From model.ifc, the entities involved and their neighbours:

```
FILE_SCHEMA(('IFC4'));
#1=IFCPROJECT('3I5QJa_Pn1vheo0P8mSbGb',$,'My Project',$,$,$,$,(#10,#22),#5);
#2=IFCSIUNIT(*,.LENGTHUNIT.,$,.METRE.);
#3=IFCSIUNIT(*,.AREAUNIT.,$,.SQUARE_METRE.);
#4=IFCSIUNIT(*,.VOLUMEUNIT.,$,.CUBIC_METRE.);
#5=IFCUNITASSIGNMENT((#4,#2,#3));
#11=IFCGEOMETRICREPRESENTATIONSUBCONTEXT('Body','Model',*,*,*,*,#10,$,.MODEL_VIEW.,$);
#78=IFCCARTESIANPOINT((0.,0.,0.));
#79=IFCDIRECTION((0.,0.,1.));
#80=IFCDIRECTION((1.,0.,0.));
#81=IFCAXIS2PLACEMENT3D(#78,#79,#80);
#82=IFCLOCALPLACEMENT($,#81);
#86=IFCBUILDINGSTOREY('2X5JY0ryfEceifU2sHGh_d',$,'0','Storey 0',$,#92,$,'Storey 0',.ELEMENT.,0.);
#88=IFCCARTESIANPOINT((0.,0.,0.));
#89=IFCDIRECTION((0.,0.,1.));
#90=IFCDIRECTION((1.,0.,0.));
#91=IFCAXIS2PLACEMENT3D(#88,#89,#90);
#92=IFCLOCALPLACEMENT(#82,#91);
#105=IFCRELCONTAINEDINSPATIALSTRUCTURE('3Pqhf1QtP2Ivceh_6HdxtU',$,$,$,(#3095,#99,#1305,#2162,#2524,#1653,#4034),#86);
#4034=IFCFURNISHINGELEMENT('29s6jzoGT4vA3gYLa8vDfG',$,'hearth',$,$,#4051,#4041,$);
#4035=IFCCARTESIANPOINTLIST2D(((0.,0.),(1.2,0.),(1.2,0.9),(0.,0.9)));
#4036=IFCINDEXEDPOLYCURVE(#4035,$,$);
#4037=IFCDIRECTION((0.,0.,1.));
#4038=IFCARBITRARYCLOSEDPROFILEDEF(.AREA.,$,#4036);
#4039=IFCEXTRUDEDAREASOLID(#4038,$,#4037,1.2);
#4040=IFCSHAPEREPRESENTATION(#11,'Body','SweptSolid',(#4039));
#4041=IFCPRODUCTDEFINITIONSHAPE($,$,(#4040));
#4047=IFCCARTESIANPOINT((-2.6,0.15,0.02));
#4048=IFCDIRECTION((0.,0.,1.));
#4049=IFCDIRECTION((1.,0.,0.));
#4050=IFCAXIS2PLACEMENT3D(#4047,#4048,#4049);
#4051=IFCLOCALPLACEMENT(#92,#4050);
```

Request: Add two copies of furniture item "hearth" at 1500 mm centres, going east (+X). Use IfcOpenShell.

```python
import numpy as np
import ifcopenshell
import ifcopenshell.api.geometry
import ifcopenshell.api.root
import ifcopenshell.util.element
import ifcopenshell.util.placement
import ifcopenshell.util.unit

model = ifcopenshell.open("model.ifc")
unit_scale = ifcopenshell.util.unit.calculate_unit_scale(model)

source = model.by_guid("29s6jzoGT4vA3gYLa8vDfG")
base = ifcopenshell.util.placement.get_local_placement(source.ObjectPlacement)
step = np.array([1.0, 0.0, 0.0]) * 1.5 / unit_scale

for i in range(1, 3):
    copy = ifcopenshell.api.root.copy_class(model, product=source)
    copy.Representation = ifcopenshell.util.element.copy_deep(
        model, source.Representation, exclude=["IfcGeometricRepresentationContext", "IfcRepresentationMap"]
    )
    matrix = base.copy()
    matrix[:3, 3] += i * step
    print("added at", matrix[:3, 3].round(3) + 0.0)
    ifcopenshell.api.geometry.edit_object_placement(model, product=copy, matrix=matrix, is_si=False)

model.write("model_edited.ifc")
```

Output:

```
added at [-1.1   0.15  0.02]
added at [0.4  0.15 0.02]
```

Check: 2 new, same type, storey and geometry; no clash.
